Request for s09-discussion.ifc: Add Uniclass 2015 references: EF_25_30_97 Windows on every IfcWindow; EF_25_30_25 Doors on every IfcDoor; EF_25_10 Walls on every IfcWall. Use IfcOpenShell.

First a look at what the model holds.

```python
import ifcopenshell

model = ifcopenshell.open("s09-discussion.ifc")
print(model.schema)
print("classifications:", [c.Name for c in model.by_type("IfcClassification")])
for ifc_class in ("IfcDoor", "IfcRoof", "IfcStair", "IfcWall", "IfcWindow"):
    print(ifc_class, len(model.by_type(ifc_class)))
```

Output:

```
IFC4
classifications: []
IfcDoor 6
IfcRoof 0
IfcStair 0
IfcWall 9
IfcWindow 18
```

```python
import ifcopenshell
import ifcopenshell.api.classification

model = ifcopenshell.open("s09-discussion.ifc")

system = ifcopenshell.api.classification.add_classification(model, classification="Uniclass 2015")

codes = {
    "IfcWindow": ("EF_25_30_97", "Windows"),
    "IfcDoor": ("EF_25_30_25", "Doors"),
    "IfcWall": ("EF_25_10", "Walls"),
}
for ifc_class, (code, name) in codes.items():
    products = model.by_type(ifc_class)
    ifcopenshell.api.classification.add_reference(
        model, products=products, classification=system, identification=code, name=name
    )
    print(code, len(products))

model.write("s09-discussion_updated.ifc")
```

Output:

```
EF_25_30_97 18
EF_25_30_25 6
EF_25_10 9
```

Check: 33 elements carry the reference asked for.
